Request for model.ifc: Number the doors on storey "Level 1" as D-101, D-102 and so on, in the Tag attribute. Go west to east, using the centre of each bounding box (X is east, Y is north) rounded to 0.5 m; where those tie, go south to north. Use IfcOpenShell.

First a look at what the model holds.

```python
import ifcopenshell
import ifcopenshell.util.element
import ifcopenshell.util.placement

model = ifcopenshell.open("model.ifc")
print(model.schema)
storey = next(s for s in model.by_type("IfcBuildingStorey") if s.Name == "Level 1")
doors = [e for e in ifcopenshell.util.element.get_decomposition(storey) if e.is_a("IfcDoor")]
for e in sorted(doors, key=lambda e: e.id()):
    origin = ifcopenshell.util.placement.get_local_placement(e.ObjectPlacement)[:3, 3]
    print(e.id(), e.Tag, e.Name, origin.round(2) + 0.0, sep=" | ")
```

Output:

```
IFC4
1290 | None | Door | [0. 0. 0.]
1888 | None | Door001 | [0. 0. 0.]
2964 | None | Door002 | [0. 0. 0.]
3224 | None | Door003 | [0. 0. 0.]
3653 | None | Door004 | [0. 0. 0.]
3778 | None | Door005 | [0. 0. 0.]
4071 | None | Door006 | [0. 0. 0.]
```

```python
import ifcopenshell
import ifcopenshell.geom
import ifcopenshell.util.element
import ifcopenshell.util.shape

model = ifcopenshell.open("model.ifc")
settings = ifcopenshell.geom.settings()
settings.set("use-world-coords", True)


def centre(element):
    shape = ifcopenshell.geom.create_shape(settings, element)
    return ifcopenshell.util.shape.get_bbox_centroid(shape.geometry)


storey = next(s for s in model.by_type("IfcBuildingStorey") if s.Name == "Level 1")
doors = [e for e in ifcopenshell.util.element.get_decomposition(storey) if e.is_a("IfcDoor")]

# Insertion points can sit at a corner or the storey origin, so sort by the geometry (in metres).
centres = {e: centre(e) for e in doors}
doors.sort(key=lambda e: (round(centres[e][0] / 0.5), centres[e][1]))

for i, e in enumerate(doors, start=1):
    number = f"D-1{i:02d}"
    e.Tag = number
    print(e.id(), number)

model.write("model-out.ifc")
```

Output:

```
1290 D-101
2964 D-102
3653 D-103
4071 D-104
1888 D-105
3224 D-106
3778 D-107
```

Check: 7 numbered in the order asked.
